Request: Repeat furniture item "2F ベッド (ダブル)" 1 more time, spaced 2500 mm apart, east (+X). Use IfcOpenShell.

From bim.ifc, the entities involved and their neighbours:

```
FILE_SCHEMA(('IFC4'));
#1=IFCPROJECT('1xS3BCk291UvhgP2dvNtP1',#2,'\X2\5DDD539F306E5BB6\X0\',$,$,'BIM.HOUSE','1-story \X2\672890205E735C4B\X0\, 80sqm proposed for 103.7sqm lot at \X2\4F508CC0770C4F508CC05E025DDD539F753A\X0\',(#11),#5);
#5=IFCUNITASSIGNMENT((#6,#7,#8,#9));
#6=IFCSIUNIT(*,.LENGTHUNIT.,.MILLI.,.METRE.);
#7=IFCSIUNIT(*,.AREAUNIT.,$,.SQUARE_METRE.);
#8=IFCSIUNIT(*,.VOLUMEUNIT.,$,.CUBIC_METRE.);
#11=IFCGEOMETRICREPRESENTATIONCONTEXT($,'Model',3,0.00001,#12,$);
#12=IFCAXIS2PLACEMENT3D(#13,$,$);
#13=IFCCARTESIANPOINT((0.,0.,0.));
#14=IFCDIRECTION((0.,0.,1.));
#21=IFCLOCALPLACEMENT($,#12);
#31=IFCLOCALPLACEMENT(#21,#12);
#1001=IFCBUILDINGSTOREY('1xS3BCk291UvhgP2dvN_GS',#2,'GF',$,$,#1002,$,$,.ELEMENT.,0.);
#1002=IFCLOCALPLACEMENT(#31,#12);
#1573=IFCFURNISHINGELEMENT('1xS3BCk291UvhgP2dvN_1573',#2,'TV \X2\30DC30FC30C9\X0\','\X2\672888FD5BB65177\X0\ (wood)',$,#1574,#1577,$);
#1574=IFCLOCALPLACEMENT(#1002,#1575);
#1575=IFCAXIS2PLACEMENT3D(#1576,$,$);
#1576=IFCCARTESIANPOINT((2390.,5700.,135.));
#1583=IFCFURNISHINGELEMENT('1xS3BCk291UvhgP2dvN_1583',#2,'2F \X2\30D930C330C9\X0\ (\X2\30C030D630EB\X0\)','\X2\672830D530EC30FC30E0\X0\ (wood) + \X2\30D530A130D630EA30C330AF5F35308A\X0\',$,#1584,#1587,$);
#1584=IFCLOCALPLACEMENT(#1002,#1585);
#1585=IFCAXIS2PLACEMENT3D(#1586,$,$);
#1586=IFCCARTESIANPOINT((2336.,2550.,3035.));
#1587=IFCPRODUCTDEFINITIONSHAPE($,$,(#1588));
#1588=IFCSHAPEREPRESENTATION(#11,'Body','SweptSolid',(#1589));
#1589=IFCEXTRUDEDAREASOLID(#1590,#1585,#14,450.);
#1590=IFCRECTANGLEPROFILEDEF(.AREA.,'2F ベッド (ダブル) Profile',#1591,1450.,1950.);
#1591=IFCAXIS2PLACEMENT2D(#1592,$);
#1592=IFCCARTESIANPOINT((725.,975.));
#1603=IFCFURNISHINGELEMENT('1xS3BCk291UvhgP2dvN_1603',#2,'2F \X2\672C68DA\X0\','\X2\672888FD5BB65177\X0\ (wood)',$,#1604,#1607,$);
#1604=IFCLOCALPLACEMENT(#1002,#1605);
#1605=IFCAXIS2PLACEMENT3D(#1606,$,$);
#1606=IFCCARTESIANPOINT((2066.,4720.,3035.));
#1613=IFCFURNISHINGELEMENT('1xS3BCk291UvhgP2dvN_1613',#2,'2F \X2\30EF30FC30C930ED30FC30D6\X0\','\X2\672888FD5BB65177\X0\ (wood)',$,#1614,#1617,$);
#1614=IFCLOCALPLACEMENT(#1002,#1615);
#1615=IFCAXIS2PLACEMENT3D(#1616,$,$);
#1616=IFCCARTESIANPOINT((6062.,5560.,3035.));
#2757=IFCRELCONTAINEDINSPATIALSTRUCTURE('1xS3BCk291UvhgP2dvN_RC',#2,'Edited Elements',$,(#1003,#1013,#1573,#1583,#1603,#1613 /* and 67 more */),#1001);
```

```python
import numpy as np
import ifcopenshell
import ifcopenshell.api.geometry
import ifcopenshell.api.root
import ifcopenshell.util.element
import ifcopenshell.util.placement

model = ifcopenshell.open("bim.ifc")


def reuse_history(source, copy):
    """copy_class also copies each property set's owner history, people and application; keep the originals."""
    for rel in copy.IsDefinedBy:
        if rel.is_a("IfcRelDefinesByProperties") and (history := rel.RelatingPropertyDefinition.OwnerHistory):
            rel.RelatingPropertyDefinition.OwnerHistory = source.OwnerHistory
            ifcopenshell.util.element.remove_deep2(model, history)


source = model.by_id(1583)
base = ifcopenshell.util.placement.get_local_placement(source.ObjectPlacement)
step = np.array([1.0, 0.0, 0.0]) * 2500.0

for i in range(1, 2):
    copy = ifcopenshell.api.root.copy_class(model, product=source)
    copy.Representation = ifcopenshell.util.element.copy_deep(
        model, source.Representation, exclude=["IfcGeometricRepresentationContext", "IfcRepresentationMap"]
    )
    reuse_history(source, copy)
    matrix = base.copy()
    matrix[:3, 3] += i * step
    print("added at", matrix[:3, 3].round(3) + 0.0)
    ifcopenshell.api.geometry.edit_object_placement(model, product=copy, matrix=matrix, is_si=False)

model.write("bim_rev.ifc")
```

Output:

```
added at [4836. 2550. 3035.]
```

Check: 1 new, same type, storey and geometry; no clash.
